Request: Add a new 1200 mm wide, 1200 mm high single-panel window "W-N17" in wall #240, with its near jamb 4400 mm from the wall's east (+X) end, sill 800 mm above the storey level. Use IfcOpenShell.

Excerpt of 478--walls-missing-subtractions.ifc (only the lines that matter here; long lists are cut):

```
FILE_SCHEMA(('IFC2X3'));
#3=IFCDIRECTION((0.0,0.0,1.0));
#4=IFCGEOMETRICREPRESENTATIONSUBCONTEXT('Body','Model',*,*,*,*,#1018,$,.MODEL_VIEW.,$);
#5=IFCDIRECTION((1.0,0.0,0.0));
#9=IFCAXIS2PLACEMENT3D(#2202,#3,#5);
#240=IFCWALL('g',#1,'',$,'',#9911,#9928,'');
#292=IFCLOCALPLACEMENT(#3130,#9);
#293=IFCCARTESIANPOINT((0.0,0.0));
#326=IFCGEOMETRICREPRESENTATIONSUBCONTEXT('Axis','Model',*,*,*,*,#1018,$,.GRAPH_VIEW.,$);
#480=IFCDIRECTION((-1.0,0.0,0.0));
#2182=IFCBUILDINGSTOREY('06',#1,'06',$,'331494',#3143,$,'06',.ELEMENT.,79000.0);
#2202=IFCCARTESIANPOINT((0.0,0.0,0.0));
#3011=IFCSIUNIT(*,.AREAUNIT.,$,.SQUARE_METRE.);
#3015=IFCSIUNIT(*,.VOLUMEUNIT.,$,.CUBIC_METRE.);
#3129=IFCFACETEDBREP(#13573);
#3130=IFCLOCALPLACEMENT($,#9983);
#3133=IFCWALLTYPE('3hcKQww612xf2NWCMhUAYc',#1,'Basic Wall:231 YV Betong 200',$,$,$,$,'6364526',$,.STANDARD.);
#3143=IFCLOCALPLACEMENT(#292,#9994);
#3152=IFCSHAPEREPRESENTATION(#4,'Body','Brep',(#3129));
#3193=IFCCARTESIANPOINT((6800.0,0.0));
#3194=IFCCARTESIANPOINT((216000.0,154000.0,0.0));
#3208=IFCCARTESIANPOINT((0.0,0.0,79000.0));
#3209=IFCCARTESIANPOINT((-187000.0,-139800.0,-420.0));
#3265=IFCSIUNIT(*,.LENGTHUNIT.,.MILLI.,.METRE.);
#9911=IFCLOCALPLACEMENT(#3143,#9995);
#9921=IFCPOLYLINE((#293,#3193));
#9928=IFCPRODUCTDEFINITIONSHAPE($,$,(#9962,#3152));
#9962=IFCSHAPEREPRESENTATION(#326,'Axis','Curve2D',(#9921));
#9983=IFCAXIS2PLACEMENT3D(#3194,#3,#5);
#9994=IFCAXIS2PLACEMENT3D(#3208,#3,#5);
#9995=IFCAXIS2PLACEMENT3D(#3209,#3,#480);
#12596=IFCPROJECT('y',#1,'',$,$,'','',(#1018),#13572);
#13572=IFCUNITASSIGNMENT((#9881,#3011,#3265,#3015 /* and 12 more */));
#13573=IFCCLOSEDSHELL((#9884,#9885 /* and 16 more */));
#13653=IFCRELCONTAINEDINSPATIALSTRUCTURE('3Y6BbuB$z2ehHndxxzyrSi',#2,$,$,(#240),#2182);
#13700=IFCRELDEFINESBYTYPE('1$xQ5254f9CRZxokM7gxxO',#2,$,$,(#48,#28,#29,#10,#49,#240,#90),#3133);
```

```python
import numpy as np
import ifcopenshell
import ifcopenshell.api.feature
import ifcopenshell.api.geometry
import ifcopenshell.api.root
import ifcopenshell.api.spatial
import ifcopenshell.api.type
import ifcopenshell.geom
import ifcopenshell.util.element
import ifcopenshell.util.placement
import ifcopenshell.util.representation
import ifcopenshell.util.shape
import ifcopenshell.util.unit

model = ifcopenshell.open("478--walls-missing-subtractions.ifc")
unit_scale = ifcopenshell.util.unit.calculate_unit_scale(model)
settings = ifcopenshell.geom.settings()


def volume(element):
    """Net volume in cubic metres, openings subtracted."""
    shape = ifcopenshell.geom.create_shape(settings, element)
    return ifcopenshell.util.shape.get_volume(shape.geometry)


wall = model.by_guid("g")
storey = ifcopenshell.util.element.get_container(wall, ifc_class="IfcBuildingStorey")
context = ifcopenshell.util.representation.get_context(model, "Model", "Body", "MODEL_VIEW")
before = volume(wall)

width, height, from_end, sill = 1.2, 1.2, 4.4, 0.8  # metres

# The wall runs along its own X axis, and the end named is its -X end.
wall_shape = ifcopenshell.geom.create_shape(settings, wall)
x, y, z = ifcopenshell.util.shape.get_vertices(wall_shape.geometry).T
start = x.min() + from_end
face, thickness = float(y.min()), float(y.max() - y.min())
wall_matrix = ifcopenshell.util.placement.get_local_placement(wall.ObjectPlacement)
level = ifcopenshell.util.placement.get_local_placement(storey.ObjectPlacement)[2, 3]


def in_wall(x, y):
    """Placement at x, y metres in the wall's axes, at sill height."""
    matrix = wall_matrix.copy()
    matrix[:, 3] = wall_matrix @ np.array([x / unit_scale, y / unit_scale, 0.0, 1.0])
    matrix[2, 3] = level + sill / unit_scale
    return matrix


# Opening: a box that overshoots both wall faces by 50 mm.
opening = ifcopenshell.api.root.create_entity(model, ifc_class="IfcOpeningElement")
box = ifcopenshell.api.geometry.add_wall_representation(
    model, context=context, length=width, height=height, thickness=thickness + 0.1
)
ifcopenshell.api.geometry.assign_representation(model, product=opening, representation=box)
ifcopenshell.api.geometry.edit_object_placement(model, product=opening, matrix=in_wall(start, face - 0.05), is_si=False)
ifcopenshell.api.feature.add_feature(model, feature=opening, element=wall)

window = ifcopenshell.api.root.create_entity(model, ifc_class="IfcWindow", name="W-N17")
window.OverallWidth, window.OverallHeight = width / unit_scale, height / unit_scale
body = ifcopenshell.api.geometry.add_window_representation(
    model,
    context=context,
    overall_width=window.OverallWidth,
    overall_height=window.OverallHeight,
    partition_type="SINGLE_PANEL",
)
ifcopenshell.api.geometry.assign_representation(model, product=window, representation=body)
ifcopenshell.api.spatial.assign_container(model, products=[window], relating_structure=storey)
fills = ifcopenshell.api.feature.add_filling(model, opening=opening, element=window)
fills.OwnerHistory = window.OwnerHistory  # required in IFC2X3

# IFC2X3 keeps the operation on the window style.
style = ifcopenshell.api.root.create_entity(model, ifc_class="IfcWindowStyle", name="W-N17")
style.OperationType, style.ConstructionType = "SINGLE_PANEL", "NOTDEFINED"
style.ParameterTakesPrecedence = style.Sizeable = False
ifcopenshell.api.type.assign_type(model, related_objects=[window], relating_type=style)

# Centre the window in the wall's thickness.
ifcopenshell.api.geometry.edit_object_placement(model, product=window, matrix=in_wall(start, face), is_si=False)
window_shape = ifcopenshell.geom.create_shape(settings, window)
depth = ifcopenshell.util.shape.get_vertices(window_shape.geometry)[:, 1]
offset = face + thickness / 2 - (depth.min() + depth.max()) / 2
ifcopenshell.api.geometry.edit_object_placement(model, product=window, matrix=in_wall(start, offset), is_si=False)

after = volume(wall)

print(f"wall volume {before:.3f} -> {after:.3f} m3")

model.write("478--walls-missing-subtractions_v2.ifc")
```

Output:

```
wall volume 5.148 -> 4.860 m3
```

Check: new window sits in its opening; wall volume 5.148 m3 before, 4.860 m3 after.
